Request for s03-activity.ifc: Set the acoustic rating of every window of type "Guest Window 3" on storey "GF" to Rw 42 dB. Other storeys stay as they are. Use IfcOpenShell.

First a look at what the model holds.

```python
import ifcopenshell
import ifcopenshell.util.element

model = ifcopenshell.open("s03-activity.ifc")
print(model.schema)
storey = next(s for s in model.by_type("IfcBuildingStorey") if s.Name == "GF")
windows = [e for e in ifcopenshell.util.element.get_decomposition(storey) if e.is_a("IfcWindow")]
seen = {}
for e in windows:
    element_type = ifcopenshell.util.element.get_type(e)
    key = (element_type.Name if element_type != e and element_type else None, ifcopenshell.util.element.get_pset(e, "Pset_WindowCommon", "AcousticRating"))
    seen[key] = seen.get(key, 0) + 1
for (name, value), count in sorted(seen.items(), key=str):
    print(count, "x", name, "|", value)
```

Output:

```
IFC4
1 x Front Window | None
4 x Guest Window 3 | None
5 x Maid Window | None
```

```python
import ifcopenshell
import ifcopenshell.api.pset
import ifcopenshell.util.element

model = ifcopenshell.open("s03-activity.ifc")

storey = next(s for s in model.by_type("IfcBuildingStorey") if s.Name == "GF")
windows = [e for e in ifcopenshell.util.element.get_decomposition(storey) if e.is_a("IfcWindow")]

count = 0
for e in windows:
    element_type = ifcopenshell.util.element.get_type(e)
    if element_type in (None, e) or element_type.Name != "Guest Window 3":
        continue
    # add_pset returns the element's existing set when there is one.
    pset = ifcopenshell.api.pset.add_pset(model, product=e, name="Pset_WindowCommon")
    ifcopenshell.api.pset.edit_pset(model, pset=pset, properties={"AcousticRating": "Rw 42 dB"})
    count += 1

print(count, "windows updated")

model.write("s03-activity_edited.ifc")
```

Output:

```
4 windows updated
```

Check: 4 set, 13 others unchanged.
